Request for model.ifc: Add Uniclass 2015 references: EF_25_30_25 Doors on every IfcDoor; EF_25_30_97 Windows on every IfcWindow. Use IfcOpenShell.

First a look at what the model holds.

```python
import ifcopenshell

model = ifcopenshell.open("model.ifc")
print(model.schema)
print("classifications:", [c.Name for c in model.by_type("IfcClassification")])
for ifc_class in ("IfcDoor", "IfcRoof", "IfcStair", "IfcWall", "IfcWindow"):
    print(ifc_class, len(model.by_type(ifc_class)))
```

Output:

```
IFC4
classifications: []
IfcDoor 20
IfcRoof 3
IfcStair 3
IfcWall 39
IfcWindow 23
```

```python
import ifcopenshell
import ifcopenshell.api.classification

model = ifcopenshell.open("model.ifc")

system = ifcopenshell.api.classification.add_classification(model, classification="Uniclass 2015")

codes = {
    "IfcDoor": ("EF_25_30_25", "Doors"),
    "IfcWindow": ("EF_25_30_97", "Windows"),
}
for ifc_class, (code, name) in codes.items():
    products = model.by_type(ifc_class)
    ifcopenshell.api.classification.add_reference(
        model, products=products, classification=system, identification=code, name=name
    )
    print(code, len(products))

model.write("model_updated.ifc")
```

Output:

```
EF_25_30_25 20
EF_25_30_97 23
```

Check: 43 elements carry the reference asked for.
